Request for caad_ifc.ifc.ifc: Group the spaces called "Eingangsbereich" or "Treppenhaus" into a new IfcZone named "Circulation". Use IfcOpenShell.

First a look at what the model holds.

```python
import ifcopenshell

model = ifcopenshell.open("caad_ifc.ifc.ifc")
print(model.schema)
seen = {}
for space in model.by_type("IfcSpace"):
    seen[space.LongName] = seen.get(space.LongName, 0) + 1
for name, count in sorted(seen.items(), key=str):
    print(count, "x", name)
print("zones:", [z.Name for z in model.by_type("IfcZone")][:20])
```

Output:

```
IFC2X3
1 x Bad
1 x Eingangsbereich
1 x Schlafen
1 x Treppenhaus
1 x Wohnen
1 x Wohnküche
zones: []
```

```python
import ifcopenshell
import ifcopenshell.api.group
import ifcopenshell.api.root

model = ifcopenshell.open("caad_ifc.ifc.ifc")

names = {"Eingangsbereich", "Treppenhaus"}
spaces = [s for s in model.by_type("IfcSpace") if s.LongName in names]

zone = ifcopenshell.api.root.create_entity(model, ifc_class="IfcZone", name="Circulation")
ifcopenshell.api.group.assign_group(model, products=spaces, group=zone)
print(len(spaces), "spaces in", zone.Name)

model.write("caad_ifc.ifc_edited.ifc")
```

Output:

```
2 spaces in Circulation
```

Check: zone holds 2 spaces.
